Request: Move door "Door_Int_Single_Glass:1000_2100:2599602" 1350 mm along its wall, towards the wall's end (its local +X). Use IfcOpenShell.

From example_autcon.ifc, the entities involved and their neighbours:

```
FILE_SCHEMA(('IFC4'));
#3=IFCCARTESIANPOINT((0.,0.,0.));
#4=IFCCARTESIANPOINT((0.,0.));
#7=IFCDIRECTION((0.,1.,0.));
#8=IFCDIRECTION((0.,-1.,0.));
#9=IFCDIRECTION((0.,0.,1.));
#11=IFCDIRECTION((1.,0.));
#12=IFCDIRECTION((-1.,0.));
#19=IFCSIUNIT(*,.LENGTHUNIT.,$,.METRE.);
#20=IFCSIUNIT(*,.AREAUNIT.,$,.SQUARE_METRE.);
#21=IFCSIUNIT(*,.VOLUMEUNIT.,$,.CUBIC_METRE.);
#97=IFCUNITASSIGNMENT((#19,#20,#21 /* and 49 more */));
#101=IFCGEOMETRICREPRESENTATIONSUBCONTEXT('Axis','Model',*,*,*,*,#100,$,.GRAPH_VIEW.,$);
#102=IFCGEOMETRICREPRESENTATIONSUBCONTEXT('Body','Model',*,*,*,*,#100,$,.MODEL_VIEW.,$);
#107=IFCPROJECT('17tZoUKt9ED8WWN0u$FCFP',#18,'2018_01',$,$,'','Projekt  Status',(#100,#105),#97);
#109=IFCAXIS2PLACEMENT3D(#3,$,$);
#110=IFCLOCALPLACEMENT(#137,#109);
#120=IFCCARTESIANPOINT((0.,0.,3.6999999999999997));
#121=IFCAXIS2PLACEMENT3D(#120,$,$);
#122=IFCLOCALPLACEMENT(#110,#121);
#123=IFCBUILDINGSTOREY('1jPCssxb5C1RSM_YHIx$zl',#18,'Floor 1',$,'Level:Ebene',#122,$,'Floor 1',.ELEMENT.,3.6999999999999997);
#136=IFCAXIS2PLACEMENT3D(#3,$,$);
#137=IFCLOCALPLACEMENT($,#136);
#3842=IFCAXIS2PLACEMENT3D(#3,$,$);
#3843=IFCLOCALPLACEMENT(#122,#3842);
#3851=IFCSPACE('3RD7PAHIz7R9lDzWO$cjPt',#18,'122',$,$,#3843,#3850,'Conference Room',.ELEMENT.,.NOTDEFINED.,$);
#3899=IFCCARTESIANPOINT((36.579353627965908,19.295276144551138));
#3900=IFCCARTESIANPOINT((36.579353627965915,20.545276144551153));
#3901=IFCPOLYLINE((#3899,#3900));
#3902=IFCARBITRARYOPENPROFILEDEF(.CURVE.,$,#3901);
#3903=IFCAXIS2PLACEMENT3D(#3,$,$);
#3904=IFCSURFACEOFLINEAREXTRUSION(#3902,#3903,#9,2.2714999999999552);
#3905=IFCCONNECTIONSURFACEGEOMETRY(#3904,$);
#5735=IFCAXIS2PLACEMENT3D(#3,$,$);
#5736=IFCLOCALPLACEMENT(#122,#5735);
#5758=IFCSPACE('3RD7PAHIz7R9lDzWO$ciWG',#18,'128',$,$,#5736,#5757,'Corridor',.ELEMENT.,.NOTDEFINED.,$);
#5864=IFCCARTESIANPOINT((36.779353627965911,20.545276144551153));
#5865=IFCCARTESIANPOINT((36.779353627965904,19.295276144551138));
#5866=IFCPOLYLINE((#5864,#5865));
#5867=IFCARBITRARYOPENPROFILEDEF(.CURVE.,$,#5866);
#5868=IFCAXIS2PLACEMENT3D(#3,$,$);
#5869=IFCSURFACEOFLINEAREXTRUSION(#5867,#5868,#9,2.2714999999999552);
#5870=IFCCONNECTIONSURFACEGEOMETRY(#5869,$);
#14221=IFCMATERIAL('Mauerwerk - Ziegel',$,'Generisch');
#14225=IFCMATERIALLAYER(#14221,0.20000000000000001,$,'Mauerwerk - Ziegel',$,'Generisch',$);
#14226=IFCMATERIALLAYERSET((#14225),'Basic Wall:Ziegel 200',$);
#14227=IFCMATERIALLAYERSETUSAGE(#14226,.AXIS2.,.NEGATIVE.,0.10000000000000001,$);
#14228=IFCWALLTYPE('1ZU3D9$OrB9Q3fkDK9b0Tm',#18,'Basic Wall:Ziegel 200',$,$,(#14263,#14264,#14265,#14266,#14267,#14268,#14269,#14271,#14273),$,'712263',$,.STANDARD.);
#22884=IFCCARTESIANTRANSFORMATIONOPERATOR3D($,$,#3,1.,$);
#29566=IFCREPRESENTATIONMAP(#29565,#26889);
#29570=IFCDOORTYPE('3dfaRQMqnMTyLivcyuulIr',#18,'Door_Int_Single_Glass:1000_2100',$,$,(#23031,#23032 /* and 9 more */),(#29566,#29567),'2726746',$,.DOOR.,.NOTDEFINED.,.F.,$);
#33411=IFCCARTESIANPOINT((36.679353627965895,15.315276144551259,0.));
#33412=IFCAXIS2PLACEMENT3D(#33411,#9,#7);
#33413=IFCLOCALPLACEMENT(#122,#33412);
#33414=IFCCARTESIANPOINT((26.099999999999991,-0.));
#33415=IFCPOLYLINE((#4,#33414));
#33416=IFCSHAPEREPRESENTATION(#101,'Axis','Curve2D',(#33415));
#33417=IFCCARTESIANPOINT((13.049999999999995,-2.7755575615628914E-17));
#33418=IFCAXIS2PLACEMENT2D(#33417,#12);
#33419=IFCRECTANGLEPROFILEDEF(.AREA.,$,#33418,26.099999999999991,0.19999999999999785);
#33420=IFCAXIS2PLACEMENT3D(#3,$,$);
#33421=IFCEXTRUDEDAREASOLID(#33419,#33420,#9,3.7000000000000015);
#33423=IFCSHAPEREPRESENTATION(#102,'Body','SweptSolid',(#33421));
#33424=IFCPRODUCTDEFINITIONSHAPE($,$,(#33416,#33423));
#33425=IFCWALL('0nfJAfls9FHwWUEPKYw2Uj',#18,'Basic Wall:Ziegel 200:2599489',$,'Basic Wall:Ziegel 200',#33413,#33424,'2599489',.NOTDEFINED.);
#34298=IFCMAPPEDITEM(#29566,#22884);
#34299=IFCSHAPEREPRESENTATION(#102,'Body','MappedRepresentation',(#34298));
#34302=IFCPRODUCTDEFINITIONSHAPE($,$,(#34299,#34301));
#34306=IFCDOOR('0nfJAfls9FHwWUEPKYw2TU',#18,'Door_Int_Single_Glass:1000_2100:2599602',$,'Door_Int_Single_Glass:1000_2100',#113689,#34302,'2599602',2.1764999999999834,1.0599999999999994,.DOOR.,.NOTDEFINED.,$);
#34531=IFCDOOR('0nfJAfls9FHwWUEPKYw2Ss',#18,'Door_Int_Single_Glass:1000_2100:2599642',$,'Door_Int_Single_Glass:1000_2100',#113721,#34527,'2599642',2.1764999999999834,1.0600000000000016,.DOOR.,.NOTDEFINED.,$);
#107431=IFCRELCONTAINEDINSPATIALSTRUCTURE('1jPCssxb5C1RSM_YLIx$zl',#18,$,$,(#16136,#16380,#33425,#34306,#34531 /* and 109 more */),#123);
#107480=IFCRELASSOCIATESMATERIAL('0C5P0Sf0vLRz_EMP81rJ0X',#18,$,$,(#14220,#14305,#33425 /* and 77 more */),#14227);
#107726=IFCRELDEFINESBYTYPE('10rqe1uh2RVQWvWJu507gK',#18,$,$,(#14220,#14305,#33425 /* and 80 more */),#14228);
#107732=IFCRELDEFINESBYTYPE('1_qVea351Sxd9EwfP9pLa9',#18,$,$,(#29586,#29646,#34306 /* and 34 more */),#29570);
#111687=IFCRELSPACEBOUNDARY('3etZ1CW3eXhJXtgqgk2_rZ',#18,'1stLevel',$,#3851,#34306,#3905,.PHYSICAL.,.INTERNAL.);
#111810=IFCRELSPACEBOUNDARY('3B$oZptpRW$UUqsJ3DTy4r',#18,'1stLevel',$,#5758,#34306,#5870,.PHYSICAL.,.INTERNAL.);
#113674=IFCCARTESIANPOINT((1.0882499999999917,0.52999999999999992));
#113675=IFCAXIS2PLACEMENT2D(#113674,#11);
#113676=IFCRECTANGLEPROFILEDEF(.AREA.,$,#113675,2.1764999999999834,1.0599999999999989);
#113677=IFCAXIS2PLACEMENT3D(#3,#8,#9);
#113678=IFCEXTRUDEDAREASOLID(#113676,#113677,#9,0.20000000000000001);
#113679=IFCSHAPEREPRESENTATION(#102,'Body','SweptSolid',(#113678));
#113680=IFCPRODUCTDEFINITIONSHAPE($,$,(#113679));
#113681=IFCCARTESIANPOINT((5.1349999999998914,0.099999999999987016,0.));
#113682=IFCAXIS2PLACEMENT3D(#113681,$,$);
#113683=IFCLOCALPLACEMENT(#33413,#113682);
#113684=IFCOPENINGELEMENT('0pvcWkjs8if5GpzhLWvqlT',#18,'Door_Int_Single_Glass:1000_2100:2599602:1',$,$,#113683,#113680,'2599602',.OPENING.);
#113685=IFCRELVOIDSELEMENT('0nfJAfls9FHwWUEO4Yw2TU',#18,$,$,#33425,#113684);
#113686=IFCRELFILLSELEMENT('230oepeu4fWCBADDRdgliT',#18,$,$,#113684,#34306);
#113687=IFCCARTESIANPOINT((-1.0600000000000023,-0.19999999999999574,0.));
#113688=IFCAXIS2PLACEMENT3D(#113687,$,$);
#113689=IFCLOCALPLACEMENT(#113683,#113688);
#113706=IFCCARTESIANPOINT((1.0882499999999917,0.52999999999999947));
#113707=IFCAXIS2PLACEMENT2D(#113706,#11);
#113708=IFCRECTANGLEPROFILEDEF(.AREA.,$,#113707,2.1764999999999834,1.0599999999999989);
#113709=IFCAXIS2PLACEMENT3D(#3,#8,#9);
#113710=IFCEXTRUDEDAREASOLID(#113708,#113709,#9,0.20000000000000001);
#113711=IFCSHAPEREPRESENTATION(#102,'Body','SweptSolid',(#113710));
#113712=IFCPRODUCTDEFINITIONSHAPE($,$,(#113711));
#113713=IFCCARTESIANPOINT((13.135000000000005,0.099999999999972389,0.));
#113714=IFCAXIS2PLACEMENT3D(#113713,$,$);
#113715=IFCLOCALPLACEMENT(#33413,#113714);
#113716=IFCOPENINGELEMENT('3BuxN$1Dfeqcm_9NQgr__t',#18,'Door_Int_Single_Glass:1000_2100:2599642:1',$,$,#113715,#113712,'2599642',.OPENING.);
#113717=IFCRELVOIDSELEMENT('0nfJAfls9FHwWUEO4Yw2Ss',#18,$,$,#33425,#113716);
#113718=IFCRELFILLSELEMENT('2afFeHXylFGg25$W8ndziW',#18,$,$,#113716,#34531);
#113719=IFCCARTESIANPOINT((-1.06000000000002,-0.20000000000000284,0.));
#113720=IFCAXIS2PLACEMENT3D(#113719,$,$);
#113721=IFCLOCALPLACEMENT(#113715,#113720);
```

```python
import numpy as np
import ifcopenshell
import ifcopenshell.api.geometry
import ifcopenshell.util.placement
import ifcopenshell.util.unit

model = ifcopenshell.open("example_autcon.ifc")
unit_scale = ifcopenshell.util.unit.calculate_unit_scale(model)

door = model.by_id(34306)
opening = door.FillsVoids[0].RelatingOpeningElement
wall = opening.VoidsElements[0].RelatingBuildingElement

wall_matrix = ifcopenshell.util.placement.get_local_placement(wall.ObjectPlacement)
shift = wall_matrix[:3, 0] * 1.35 / unit_scale
before = ifcopenshell.util.placement.get_local_placement(door.ObjectPlacement)[:3, 3].copy()

# The door is placed relative to its opening, so it follows when the opening moves.
matrix = ifcopenshell.util.placement.get_local_placement(opening.ObjectPlacement)
matrix[:3, 3] += shift
ifcopenshell.api.geometry.edit_object_placement(
    model, product=opening, matrix=matrix, is_si=False, should_transform_children=True
)

# Space boundary surfaces are stored in each space's coordinates; move them too.
for rel in door.ProvidesBoundaries:
    if not rel.ConnectionGeometry:
        continue
    surface = rel.ConnectionGeometry.SurfaceOnRelatingElement
    space_matrix = ifcopenshell.util.placement.get_local_placement(rel.RelatingSpace.ObjectPlacement)
    point = np.array(surface.Position.Location.Coordinates) + space_matrix[:3, :3].T @ shift
    surface.Position = model.createIfcAxis2Placement3D(
        model.createIfcCartesianPoint(point.tolist()), surface.Position.Axis, surface.Position.RefDirection
    )

after = ifcopenshell.util.placement.get_local_placement(door.ObjectPlacement)[:3, 3]
print("door moved by", (after - before).round(3) + 0.0)

model.write("example_autcon-out.ifc")
```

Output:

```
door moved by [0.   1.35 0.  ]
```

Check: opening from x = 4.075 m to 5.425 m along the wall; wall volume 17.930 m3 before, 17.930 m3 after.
